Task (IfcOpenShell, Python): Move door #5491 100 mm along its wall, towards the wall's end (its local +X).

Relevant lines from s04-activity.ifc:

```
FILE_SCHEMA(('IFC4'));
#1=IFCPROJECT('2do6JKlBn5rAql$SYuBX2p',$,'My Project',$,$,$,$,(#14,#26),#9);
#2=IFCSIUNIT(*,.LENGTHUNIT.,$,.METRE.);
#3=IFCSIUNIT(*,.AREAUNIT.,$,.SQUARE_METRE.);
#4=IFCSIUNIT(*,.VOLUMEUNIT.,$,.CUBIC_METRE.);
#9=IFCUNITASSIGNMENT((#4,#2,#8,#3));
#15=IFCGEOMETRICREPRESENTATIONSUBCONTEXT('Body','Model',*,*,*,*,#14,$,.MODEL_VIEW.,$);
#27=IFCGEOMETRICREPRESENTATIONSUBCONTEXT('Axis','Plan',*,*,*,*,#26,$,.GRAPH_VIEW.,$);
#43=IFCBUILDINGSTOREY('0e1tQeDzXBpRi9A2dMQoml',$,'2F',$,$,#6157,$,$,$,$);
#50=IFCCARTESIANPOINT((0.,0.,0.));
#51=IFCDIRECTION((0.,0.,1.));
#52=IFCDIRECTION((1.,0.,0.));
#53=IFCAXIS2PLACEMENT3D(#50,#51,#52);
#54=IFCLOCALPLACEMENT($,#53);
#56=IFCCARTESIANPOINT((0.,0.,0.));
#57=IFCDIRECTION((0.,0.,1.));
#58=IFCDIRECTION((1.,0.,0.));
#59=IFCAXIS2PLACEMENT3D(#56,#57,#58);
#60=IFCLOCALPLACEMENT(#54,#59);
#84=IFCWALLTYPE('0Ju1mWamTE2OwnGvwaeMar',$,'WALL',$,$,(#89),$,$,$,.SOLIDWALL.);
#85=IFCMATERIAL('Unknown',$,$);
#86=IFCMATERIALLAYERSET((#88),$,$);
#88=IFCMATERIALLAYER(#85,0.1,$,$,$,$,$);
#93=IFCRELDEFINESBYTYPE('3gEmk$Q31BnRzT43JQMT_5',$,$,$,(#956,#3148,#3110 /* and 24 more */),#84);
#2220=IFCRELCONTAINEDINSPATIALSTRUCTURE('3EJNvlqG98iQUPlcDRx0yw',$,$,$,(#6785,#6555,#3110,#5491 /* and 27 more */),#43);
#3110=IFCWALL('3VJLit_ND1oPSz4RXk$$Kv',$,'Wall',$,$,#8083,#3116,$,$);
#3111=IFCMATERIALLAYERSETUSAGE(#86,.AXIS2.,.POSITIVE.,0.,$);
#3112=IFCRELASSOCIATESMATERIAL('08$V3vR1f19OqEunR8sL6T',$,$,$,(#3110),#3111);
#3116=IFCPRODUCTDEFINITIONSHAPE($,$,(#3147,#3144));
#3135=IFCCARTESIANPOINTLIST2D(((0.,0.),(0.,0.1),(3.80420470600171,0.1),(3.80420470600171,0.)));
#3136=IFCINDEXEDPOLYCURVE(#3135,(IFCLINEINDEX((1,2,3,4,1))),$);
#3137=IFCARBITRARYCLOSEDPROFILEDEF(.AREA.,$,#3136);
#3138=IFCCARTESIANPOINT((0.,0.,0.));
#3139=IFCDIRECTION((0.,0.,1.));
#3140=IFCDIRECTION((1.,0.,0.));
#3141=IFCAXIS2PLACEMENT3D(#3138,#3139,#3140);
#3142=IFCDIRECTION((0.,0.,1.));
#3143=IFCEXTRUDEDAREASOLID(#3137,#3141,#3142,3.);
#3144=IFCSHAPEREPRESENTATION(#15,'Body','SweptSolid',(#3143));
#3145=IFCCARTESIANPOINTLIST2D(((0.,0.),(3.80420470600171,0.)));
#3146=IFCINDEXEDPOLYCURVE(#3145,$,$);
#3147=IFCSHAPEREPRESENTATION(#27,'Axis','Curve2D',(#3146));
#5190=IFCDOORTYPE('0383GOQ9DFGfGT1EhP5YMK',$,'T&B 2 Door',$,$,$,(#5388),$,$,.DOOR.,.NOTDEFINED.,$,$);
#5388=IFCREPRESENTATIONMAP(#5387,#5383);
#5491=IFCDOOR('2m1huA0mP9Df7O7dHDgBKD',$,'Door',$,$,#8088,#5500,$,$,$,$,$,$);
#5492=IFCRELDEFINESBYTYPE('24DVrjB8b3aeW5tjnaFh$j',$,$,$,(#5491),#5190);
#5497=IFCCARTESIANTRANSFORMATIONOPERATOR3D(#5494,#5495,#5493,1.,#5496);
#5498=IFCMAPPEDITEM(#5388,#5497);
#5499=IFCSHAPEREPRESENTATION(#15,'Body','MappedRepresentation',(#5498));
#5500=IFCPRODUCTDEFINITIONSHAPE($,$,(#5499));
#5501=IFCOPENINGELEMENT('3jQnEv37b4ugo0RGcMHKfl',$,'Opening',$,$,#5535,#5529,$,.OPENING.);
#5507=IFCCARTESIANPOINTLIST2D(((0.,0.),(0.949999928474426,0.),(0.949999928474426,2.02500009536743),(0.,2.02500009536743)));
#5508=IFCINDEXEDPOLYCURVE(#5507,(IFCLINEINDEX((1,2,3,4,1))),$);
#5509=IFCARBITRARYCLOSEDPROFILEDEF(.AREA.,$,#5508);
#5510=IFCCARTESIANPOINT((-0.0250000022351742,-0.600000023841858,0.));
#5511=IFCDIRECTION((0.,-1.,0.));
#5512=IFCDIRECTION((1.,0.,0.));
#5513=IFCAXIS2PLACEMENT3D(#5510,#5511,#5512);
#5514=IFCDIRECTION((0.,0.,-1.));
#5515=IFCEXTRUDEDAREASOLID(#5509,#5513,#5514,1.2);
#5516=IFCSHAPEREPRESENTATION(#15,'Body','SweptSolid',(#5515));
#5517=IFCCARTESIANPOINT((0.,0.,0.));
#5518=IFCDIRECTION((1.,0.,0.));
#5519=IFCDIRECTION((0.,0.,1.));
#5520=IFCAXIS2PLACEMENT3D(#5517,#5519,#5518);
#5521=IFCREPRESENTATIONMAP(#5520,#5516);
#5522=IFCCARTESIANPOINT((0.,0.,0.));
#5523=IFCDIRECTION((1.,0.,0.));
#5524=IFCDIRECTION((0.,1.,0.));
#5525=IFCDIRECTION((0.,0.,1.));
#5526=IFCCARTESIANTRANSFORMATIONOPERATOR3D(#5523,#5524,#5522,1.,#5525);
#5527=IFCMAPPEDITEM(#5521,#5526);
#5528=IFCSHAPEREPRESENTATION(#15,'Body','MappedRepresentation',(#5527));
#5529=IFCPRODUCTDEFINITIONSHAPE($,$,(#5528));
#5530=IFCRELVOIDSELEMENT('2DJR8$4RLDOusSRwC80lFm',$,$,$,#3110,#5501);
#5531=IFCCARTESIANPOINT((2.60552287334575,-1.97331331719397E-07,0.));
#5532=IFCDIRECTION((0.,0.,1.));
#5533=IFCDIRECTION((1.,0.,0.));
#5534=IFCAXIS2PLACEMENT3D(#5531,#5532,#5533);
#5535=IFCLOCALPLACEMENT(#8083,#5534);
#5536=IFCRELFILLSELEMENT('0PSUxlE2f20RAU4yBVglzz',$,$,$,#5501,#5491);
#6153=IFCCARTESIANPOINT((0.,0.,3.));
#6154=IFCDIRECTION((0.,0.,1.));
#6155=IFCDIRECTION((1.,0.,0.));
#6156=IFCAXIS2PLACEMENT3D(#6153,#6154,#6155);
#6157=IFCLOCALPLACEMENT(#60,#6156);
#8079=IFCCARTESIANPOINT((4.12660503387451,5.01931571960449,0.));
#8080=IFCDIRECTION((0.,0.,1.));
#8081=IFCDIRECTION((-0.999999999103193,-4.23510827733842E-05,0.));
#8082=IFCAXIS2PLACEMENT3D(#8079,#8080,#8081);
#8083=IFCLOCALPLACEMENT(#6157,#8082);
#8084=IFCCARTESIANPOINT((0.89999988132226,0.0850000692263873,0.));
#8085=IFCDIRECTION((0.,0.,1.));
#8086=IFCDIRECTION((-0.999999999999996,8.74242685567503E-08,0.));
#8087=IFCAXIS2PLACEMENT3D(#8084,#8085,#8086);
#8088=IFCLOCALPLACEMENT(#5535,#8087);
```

```python
import ifcopenshell
import ifcopenshell.api.geometry
import ifcopenshell.util.placement

model = ifcopenshell.open("s04-activity.ifc")

door = model.by_guid("2m1huA0mP9Df7O7dHDgBKD")
opening = door.FillsVoids[0].RelatingOpeningElement
wall = opening.VoidsElements[0].RelatingBuildingElement

wall_matrix = ifcopenshell.util.placement.get_local_placement(wall.ObjectPlacement)
shift = wall_matrix[:3, 0] * 0.1
before = ifcopenshell.util.placement.get_local_placement(door.ObjectPlacement)[:3, 3].copy()

# The door is placed relative to its opening, so it follows when the opening moves.
matrix = ifcopenshell.util.placement.get_local_placement(opening.ObjectPlacement)
matrix[:3, 3] += shift
ifcopenshell.api.geometry.edit_object_placement(
    model, product=opening, matrix=matrix, is_si=False, should_transform_children=True
)

after = ifcopenshell.util.placement.get_local_placement(door.ObjectPlacement)[:3, 3]
print("door moved by", (after - before).round(3) + 0.0)

model.write("s04-activity-out.ifc")
```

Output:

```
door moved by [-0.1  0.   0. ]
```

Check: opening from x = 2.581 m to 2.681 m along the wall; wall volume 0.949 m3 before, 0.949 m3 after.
